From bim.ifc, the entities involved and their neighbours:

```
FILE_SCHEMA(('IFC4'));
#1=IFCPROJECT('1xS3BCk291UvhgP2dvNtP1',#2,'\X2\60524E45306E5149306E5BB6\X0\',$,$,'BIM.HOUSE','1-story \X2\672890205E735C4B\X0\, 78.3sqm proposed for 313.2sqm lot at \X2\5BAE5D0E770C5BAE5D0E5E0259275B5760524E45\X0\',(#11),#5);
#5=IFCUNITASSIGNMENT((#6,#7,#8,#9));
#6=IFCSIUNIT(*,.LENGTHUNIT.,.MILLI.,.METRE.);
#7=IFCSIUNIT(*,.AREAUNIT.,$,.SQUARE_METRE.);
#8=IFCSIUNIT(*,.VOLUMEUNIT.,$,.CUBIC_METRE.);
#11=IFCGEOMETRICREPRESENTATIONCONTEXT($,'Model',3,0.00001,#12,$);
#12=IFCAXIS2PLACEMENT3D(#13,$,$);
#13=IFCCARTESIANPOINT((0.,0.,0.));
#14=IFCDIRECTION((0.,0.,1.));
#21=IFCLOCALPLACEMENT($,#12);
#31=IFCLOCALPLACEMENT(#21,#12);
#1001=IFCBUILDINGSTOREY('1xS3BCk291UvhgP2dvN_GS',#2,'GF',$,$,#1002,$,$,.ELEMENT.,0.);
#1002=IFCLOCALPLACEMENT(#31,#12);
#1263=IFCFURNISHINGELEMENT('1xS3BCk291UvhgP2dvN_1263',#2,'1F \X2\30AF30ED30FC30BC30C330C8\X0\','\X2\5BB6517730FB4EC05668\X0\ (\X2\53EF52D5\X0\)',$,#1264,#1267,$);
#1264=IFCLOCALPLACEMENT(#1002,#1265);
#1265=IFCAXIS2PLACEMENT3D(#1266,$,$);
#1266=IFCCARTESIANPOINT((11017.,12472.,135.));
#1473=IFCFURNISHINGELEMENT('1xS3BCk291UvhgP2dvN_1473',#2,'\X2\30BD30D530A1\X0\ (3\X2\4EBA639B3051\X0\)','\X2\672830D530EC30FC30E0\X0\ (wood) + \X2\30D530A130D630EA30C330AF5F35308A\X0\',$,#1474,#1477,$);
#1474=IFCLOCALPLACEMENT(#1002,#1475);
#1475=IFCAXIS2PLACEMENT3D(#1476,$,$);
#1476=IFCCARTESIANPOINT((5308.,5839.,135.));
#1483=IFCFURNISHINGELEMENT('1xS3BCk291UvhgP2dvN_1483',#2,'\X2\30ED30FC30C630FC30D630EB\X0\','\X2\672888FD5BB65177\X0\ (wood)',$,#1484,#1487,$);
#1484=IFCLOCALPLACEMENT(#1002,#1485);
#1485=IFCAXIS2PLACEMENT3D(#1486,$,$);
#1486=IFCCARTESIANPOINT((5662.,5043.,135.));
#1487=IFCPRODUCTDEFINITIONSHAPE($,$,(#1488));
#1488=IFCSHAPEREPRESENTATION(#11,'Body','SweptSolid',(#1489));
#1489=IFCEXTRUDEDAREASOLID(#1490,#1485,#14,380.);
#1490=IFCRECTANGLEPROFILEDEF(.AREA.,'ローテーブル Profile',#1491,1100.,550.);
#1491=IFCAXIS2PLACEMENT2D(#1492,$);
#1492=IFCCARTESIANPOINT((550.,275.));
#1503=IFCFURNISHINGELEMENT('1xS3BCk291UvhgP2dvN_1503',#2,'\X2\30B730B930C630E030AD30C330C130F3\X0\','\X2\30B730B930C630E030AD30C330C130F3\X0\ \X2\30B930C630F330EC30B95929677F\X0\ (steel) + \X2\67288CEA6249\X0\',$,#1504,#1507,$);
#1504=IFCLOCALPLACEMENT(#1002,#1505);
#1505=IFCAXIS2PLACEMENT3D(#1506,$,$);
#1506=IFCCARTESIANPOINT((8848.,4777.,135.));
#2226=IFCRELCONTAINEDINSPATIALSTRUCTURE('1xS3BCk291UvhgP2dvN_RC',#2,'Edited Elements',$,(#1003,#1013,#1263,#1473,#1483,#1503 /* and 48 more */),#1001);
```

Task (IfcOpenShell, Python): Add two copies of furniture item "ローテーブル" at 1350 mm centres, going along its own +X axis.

```python
import ifcopenshell
import ifcopenshell.api.geometry
import ifcopenshell.api.root
import ifcopenshell.util.element
import ifcopenshell.util.placement
import ifcopenshell.util.unit

model = ifcopenshell.open("bim.ifc")
unit_scale = ifcopenshell.util.unit.calculate_unit_scale(model)


def reuse_history(source, copy):
    """copy_class also copies each property set's owner history, people and application; keep the originals."""
    for rel in copy.IsDefinedBy:
        if rel.is_a("IfcRelDefinesByProperties") and (history := rel.RelatingPropertyDefinition.OwnerHistory):
            rel.RelatingPropertyDefinition.OwnerHistory = source.OwnerHistory
            ifcopenshell.util.element.remove_deep2(model, history)


source = model.by_guid("1xS3BCk291UvhgP2dvN_1483")
base = ifcopenshell.util.placement.get_local_placement(source.ObjectPlacement)
step = base[:3, 0] * 1.35 / unit_scale

for i in range(1, 3):
    copy = ifcopenshell.api.root.copy_class(model, product=source)
    copy.Representation = ifcopenshell.util.element.copy_deep(
        model, source.Representation, exclude=["IfcGeometricRepresentationContext", "IfcRepresentationMap"]
    )
    reuse_history(source, copy)
    matrix = base.copy()
    matrix[:3, 3] += i * step
    print("added at", matrix[:3, 3].round(3) + 0.0)
    ifcopenshell.api.geometry.edit_object_placement(model, product=copy, matrix=matrix, is_si=False)

model.write("bim_v2.ifc")
```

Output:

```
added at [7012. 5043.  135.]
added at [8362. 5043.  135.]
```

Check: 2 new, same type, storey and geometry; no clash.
